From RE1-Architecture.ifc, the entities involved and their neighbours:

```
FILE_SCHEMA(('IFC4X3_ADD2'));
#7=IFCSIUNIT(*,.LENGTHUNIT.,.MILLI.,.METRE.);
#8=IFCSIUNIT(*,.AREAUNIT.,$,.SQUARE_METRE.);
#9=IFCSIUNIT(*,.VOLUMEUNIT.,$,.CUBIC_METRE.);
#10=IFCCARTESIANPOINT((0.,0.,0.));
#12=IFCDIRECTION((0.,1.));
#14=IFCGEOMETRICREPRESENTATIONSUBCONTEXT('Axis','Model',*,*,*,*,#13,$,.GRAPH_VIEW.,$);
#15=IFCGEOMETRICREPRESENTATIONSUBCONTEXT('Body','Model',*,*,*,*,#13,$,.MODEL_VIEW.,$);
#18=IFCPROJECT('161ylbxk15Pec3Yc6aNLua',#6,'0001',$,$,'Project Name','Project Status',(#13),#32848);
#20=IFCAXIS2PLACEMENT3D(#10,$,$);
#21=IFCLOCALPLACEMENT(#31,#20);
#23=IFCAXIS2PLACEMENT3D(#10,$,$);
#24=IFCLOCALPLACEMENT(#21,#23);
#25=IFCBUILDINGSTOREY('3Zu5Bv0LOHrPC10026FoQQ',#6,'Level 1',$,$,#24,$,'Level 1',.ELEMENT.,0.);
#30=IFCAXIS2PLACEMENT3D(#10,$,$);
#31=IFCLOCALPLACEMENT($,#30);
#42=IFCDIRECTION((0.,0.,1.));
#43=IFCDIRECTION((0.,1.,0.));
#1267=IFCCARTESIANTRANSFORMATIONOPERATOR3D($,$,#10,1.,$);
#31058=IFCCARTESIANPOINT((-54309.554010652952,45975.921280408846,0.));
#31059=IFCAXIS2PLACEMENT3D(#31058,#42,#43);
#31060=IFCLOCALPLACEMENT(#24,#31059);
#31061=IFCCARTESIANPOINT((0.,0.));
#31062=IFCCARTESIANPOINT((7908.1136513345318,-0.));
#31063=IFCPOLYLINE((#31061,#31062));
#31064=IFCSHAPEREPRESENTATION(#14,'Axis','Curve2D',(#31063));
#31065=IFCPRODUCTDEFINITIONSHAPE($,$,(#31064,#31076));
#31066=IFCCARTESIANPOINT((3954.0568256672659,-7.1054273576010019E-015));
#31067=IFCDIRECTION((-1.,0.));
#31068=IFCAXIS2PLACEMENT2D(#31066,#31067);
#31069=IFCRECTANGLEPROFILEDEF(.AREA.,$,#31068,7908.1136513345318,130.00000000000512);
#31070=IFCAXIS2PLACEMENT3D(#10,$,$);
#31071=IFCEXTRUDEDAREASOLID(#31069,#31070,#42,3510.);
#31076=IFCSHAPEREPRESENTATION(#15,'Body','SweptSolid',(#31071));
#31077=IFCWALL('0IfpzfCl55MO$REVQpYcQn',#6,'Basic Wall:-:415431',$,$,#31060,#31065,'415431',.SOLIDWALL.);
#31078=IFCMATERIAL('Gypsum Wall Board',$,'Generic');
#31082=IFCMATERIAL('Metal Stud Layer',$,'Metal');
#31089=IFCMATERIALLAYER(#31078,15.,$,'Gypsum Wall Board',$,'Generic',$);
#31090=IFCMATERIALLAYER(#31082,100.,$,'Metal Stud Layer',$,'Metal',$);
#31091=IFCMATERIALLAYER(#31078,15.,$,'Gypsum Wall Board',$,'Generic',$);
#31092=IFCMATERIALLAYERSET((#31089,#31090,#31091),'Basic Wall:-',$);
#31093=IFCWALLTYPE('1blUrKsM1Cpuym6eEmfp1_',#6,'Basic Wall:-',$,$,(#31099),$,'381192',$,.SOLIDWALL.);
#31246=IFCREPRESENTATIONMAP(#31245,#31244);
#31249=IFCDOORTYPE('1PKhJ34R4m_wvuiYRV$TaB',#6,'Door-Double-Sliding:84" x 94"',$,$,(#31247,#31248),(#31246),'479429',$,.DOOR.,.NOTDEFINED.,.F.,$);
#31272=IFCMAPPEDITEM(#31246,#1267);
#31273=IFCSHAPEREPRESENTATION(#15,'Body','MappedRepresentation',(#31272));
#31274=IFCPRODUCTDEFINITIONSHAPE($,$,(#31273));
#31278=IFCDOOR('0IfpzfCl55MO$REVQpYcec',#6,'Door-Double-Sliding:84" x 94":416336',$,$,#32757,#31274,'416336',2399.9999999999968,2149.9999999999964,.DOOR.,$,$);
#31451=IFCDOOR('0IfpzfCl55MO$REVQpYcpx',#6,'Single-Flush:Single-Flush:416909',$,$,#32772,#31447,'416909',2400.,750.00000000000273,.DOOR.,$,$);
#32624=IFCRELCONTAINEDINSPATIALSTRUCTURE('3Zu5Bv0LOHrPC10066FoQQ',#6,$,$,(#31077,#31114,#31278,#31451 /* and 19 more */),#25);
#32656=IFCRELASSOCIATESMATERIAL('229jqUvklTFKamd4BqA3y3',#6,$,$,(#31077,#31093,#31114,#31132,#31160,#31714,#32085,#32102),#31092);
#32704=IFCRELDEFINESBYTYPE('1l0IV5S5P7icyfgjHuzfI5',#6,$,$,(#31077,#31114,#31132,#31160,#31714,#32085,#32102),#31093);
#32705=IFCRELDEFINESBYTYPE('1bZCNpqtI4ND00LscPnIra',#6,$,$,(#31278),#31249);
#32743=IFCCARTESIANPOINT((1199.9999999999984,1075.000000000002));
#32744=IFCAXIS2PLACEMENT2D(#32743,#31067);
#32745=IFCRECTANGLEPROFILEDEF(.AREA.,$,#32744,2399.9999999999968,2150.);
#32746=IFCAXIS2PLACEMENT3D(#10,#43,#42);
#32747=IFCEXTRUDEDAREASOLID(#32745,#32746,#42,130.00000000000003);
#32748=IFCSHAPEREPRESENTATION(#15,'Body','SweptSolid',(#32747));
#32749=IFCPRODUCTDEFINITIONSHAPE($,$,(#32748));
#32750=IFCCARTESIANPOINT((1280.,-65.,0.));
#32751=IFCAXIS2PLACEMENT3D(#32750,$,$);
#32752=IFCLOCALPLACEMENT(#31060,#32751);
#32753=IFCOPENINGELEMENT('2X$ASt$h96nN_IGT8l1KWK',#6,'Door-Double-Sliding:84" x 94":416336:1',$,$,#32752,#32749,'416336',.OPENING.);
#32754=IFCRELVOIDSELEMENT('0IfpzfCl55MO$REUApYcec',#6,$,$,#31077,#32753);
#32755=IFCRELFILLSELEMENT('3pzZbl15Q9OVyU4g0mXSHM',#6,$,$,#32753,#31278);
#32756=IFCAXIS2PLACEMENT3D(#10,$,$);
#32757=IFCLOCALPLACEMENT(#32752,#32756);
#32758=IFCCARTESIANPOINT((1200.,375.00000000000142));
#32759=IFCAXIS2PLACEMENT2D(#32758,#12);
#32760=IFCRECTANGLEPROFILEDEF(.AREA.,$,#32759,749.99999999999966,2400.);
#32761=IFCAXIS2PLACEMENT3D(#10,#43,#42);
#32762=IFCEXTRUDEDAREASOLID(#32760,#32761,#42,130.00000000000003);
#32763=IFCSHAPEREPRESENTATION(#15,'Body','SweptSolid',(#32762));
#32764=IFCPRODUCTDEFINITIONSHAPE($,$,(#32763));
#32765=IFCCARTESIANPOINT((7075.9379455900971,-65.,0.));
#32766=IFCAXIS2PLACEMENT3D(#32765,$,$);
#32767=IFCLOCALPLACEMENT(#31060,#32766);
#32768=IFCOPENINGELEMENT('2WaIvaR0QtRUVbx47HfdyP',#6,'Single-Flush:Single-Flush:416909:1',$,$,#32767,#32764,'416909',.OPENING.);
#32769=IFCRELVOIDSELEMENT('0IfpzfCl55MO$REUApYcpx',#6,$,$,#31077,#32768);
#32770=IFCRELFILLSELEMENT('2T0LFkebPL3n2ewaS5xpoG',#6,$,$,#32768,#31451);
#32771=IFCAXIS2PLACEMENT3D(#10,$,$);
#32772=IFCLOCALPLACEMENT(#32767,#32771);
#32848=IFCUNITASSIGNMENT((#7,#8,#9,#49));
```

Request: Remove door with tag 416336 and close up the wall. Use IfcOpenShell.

```python
import ifcopenshell
import ifcopenshell.api.feature
import ifcopenshell.api.root
import ifcopenshell.geom
import ifcopenshell.util.shape

model = ifcopenshell.open("RE1-Architecture.ifc")
settings = ifcopenshell.geom.settings()


def volume(element):
    """Net volume in cubic metres, openings subtracted."""
    shape = ifcopenshell.geom.create_shape(settings, element)
    return ifcopenshell.util.shape.get_volume(shape.geometry)


door = model.by_guid("0IfpzfCl55MO$REVQpYcec")
opening = door.FillsVoids[0].RelatingOpeningElement
wall = opening.VoidsElements[0].RelatingBuildingElement
before = volume(wall)

ifcopenshell.api.root.remove_product(model, product=door)
ifcopenshell.api.feature.remove_feature(model, feature=opening)

after = volume(wall)

print(f"wall volume {before:.3f} -> {after:.3f} m3")

model.write("RE1-Architecture_updated.ifc")
```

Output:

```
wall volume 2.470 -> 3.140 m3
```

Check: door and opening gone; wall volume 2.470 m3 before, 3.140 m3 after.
